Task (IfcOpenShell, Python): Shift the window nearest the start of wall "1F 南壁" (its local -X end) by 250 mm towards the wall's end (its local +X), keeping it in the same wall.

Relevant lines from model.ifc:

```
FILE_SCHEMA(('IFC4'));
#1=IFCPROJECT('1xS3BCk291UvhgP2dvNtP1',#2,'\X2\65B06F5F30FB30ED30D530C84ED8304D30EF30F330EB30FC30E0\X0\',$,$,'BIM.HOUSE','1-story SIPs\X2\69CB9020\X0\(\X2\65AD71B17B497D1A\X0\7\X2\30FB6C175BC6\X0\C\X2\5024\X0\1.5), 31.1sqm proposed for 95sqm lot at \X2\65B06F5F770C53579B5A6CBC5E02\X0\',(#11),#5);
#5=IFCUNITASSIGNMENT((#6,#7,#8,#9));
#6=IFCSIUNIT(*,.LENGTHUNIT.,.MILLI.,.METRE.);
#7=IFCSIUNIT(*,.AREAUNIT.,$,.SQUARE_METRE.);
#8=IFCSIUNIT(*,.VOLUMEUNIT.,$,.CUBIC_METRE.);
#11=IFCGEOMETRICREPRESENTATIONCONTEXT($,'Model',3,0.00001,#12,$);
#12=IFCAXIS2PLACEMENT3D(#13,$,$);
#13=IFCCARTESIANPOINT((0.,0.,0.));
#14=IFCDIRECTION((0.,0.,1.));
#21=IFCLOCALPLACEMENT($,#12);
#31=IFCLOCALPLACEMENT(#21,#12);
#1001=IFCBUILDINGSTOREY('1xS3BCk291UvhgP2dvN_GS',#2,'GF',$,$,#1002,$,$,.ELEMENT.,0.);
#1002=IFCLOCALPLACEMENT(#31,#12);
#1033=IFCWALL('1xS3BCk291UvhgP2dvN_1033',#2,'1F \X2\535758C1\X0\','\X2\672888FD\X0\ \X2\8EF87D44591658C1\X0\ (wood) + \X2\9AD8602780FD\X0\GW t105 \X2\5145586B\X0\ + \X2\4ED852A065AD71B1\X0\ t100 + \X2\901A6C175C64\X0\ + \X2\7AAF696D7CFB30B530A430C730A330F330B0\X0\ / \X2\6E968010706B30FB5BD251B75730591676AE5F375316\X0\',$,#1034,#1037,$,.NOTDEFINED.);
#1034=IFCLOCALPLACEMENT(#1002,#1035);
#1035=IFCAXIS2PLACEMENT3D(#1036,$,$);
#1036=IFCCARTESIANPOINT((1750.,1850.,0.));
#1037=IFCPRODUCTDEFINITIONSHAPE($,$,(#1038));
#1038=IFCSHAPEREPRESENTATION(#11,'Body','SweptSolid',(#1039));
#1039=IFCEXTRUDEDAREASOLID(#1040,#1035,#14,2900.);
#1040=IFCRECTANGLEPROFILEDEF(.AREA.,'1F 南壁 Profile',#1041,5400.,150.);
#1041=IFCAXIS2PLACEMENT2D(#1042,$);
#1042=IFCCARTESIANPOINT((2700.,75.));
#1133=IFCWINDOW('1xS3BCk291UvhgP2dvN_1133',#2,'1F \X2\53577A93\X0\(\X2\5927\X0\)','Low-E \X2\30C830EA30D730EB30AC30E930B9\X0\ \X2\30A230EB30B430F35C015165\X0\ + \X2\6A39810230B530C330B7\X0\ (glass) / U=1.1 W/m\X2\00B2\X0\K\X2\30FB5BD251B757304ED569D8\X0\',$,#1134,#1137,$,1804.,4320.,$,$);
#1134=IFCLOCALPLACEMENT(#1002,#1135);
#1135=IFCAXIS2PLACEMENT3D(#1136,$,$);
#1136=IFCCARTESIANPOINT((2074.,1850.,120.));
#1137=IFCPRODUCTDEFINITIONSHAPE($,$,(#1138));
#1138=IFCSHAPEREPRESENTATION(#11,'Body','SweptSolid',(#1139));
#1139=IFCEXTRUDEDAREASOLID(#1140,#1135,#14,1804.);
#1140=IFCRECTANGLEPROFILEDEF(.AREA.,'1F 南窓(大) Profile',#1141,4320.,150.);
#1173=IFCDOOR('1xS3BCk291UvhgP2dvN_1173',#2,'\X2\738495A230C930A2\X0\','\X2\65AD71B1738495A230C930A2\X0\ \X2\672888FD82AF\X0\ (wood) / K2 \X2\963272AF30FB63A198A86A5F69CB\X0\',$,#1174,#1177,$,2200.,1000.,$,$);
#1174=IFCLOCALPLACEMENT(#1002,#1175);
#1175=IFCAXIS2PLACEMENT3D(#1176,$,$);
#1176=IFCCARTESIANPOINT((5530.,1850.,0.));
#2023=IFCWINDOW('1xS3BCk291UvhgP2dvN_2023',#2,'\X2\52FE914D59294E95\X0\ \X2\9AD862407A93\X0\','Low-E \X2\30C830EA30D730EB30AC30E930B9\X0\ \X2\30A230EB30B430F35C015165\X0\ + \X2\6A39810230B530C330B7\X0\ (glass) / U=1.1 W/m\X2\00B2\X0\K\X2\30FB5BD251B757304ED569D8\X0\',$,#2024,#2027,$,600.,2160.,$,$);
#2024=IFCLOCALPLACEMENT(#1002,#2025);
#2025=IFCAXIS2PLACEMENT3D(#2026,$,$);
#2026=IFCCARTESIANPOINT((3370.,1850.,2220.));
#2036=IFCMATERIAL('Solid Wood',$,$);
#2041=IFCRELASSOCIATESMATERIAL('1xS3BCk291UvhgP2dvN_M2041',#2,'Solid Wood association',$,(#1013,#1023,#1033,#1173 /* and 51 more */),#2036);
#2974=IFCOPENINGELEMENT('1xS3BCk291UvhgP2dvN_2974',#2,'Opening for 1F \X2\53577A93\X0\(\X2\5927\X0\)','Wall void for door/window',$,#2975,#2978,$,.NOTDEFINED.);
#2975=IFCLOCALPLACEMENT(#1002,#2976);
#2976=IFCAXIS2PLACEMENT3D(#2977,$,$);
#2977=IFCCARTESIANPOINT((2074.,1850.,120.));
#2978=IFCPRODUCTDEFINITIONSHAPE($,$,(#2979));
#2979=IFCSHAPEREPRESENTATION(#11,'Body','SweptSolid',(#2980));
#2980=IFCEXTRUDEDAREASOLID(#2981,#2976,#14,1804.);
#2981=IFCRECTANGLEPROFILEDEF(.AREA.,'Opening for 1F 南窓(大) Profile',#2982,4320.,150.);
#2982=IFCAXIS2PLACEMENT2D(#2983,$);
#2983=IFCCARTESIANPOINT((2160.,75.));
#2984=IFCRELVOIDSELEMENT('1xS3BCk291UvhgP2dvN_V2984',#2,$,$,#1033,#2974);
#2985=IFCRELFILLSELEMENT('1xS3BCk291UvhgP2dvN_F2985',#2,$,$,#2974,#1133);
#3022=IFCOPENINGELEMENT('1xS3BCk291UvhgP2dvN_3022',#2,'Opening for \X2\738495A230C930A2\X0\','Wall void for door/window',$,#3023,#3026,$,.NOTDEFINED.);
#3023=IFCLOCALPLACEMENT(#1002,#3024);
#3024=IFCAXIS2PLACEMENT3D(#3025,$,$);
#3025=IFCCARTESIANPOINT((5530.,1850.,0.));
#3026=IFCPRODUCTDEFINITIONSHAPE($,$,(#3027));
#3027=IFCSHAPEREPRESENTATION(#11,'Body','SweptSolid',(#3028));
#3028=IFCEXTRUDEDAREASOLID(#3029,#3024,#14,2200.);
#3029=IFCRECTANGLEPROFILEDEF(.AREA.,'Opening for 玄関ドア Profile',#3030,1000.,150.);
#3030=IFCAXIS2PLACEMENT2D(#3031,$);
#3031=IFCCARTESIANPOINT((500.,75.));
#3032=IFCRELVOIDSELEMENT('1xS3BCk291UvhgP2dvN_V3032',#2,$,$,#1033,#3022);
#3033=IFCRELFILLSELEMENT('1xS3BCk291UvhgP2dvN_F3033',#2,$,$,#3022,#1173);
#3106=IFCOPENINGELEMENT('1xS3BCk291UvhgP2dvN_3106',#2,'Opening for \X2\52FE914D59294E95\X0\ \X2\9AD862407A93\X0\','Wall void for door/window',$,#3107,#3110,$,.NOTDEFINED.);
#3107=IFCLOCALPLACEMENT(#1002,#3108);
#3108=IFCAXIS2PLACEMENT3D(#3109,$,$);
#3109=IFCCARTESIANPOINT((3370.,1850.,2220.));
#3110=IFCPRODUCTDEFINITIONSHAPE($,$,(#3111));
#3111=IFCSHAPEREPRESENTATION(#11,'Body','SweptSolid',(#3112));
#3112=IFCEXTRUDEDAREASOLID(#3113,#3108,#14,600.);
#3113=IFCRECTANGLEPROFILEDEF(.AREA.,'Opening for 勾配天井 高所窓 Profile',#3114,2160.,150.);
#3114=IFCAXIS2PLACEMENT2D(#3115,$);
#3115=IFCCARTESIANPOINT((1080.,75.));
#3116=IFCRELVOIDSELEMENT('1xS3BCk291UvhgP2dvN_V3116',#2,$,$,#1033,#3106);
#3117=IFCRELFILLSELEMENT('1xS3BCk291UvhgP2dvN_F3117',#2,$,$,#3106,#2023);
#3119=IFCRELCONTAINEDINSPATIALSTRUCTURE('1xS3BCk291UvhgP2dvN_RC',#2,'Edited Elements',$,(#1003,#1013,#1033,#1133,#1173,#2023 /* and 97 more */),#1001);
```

```python
import ifcopenshell
import ifcopenshell.api.geometry
import ifcopenshell.util.placement

model = ifcopenshell.open("model.ifc")

window = model.by_guid("1xS3BCk291UvhgP2dvN_1133")
opening = window.FillsVoids[0].RelatingOpeningElement
wall = opening.VoidsElements[0].RelatingBuildingElement

wall_matrix = ifcopenshell.util.placement.get_local_placement(wall.ObjectPlacement)
shift = wall_matrix[:3, 0] * 250.0
before = ifcopenshell.util.placement.get_local_placement(window.ObjectPlacement)[:3, 3].copy()

# The window is not placed relative to its opening, so move both.
for product in (opening, window):
    matrix = ifcopenshell.util.placement.get_local_placement(product.ObjectPlacement)
    matrix[:3, 3] += shift
    ifcopenshell.api.geometry.edit_object_placement(model, product=product, matrix=matrix, is_si=False)

after = ifcopenshell.util.placement.get_local_placement(window.ObjectPlacement)[:3, 3]
print("window moved by", (after - before).round(3) + 0.0)

model.write("model_rev.ifc")
```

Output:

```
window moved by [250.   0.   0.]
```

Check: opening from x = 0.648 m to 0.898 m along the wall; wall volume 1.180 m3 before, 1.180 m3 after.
